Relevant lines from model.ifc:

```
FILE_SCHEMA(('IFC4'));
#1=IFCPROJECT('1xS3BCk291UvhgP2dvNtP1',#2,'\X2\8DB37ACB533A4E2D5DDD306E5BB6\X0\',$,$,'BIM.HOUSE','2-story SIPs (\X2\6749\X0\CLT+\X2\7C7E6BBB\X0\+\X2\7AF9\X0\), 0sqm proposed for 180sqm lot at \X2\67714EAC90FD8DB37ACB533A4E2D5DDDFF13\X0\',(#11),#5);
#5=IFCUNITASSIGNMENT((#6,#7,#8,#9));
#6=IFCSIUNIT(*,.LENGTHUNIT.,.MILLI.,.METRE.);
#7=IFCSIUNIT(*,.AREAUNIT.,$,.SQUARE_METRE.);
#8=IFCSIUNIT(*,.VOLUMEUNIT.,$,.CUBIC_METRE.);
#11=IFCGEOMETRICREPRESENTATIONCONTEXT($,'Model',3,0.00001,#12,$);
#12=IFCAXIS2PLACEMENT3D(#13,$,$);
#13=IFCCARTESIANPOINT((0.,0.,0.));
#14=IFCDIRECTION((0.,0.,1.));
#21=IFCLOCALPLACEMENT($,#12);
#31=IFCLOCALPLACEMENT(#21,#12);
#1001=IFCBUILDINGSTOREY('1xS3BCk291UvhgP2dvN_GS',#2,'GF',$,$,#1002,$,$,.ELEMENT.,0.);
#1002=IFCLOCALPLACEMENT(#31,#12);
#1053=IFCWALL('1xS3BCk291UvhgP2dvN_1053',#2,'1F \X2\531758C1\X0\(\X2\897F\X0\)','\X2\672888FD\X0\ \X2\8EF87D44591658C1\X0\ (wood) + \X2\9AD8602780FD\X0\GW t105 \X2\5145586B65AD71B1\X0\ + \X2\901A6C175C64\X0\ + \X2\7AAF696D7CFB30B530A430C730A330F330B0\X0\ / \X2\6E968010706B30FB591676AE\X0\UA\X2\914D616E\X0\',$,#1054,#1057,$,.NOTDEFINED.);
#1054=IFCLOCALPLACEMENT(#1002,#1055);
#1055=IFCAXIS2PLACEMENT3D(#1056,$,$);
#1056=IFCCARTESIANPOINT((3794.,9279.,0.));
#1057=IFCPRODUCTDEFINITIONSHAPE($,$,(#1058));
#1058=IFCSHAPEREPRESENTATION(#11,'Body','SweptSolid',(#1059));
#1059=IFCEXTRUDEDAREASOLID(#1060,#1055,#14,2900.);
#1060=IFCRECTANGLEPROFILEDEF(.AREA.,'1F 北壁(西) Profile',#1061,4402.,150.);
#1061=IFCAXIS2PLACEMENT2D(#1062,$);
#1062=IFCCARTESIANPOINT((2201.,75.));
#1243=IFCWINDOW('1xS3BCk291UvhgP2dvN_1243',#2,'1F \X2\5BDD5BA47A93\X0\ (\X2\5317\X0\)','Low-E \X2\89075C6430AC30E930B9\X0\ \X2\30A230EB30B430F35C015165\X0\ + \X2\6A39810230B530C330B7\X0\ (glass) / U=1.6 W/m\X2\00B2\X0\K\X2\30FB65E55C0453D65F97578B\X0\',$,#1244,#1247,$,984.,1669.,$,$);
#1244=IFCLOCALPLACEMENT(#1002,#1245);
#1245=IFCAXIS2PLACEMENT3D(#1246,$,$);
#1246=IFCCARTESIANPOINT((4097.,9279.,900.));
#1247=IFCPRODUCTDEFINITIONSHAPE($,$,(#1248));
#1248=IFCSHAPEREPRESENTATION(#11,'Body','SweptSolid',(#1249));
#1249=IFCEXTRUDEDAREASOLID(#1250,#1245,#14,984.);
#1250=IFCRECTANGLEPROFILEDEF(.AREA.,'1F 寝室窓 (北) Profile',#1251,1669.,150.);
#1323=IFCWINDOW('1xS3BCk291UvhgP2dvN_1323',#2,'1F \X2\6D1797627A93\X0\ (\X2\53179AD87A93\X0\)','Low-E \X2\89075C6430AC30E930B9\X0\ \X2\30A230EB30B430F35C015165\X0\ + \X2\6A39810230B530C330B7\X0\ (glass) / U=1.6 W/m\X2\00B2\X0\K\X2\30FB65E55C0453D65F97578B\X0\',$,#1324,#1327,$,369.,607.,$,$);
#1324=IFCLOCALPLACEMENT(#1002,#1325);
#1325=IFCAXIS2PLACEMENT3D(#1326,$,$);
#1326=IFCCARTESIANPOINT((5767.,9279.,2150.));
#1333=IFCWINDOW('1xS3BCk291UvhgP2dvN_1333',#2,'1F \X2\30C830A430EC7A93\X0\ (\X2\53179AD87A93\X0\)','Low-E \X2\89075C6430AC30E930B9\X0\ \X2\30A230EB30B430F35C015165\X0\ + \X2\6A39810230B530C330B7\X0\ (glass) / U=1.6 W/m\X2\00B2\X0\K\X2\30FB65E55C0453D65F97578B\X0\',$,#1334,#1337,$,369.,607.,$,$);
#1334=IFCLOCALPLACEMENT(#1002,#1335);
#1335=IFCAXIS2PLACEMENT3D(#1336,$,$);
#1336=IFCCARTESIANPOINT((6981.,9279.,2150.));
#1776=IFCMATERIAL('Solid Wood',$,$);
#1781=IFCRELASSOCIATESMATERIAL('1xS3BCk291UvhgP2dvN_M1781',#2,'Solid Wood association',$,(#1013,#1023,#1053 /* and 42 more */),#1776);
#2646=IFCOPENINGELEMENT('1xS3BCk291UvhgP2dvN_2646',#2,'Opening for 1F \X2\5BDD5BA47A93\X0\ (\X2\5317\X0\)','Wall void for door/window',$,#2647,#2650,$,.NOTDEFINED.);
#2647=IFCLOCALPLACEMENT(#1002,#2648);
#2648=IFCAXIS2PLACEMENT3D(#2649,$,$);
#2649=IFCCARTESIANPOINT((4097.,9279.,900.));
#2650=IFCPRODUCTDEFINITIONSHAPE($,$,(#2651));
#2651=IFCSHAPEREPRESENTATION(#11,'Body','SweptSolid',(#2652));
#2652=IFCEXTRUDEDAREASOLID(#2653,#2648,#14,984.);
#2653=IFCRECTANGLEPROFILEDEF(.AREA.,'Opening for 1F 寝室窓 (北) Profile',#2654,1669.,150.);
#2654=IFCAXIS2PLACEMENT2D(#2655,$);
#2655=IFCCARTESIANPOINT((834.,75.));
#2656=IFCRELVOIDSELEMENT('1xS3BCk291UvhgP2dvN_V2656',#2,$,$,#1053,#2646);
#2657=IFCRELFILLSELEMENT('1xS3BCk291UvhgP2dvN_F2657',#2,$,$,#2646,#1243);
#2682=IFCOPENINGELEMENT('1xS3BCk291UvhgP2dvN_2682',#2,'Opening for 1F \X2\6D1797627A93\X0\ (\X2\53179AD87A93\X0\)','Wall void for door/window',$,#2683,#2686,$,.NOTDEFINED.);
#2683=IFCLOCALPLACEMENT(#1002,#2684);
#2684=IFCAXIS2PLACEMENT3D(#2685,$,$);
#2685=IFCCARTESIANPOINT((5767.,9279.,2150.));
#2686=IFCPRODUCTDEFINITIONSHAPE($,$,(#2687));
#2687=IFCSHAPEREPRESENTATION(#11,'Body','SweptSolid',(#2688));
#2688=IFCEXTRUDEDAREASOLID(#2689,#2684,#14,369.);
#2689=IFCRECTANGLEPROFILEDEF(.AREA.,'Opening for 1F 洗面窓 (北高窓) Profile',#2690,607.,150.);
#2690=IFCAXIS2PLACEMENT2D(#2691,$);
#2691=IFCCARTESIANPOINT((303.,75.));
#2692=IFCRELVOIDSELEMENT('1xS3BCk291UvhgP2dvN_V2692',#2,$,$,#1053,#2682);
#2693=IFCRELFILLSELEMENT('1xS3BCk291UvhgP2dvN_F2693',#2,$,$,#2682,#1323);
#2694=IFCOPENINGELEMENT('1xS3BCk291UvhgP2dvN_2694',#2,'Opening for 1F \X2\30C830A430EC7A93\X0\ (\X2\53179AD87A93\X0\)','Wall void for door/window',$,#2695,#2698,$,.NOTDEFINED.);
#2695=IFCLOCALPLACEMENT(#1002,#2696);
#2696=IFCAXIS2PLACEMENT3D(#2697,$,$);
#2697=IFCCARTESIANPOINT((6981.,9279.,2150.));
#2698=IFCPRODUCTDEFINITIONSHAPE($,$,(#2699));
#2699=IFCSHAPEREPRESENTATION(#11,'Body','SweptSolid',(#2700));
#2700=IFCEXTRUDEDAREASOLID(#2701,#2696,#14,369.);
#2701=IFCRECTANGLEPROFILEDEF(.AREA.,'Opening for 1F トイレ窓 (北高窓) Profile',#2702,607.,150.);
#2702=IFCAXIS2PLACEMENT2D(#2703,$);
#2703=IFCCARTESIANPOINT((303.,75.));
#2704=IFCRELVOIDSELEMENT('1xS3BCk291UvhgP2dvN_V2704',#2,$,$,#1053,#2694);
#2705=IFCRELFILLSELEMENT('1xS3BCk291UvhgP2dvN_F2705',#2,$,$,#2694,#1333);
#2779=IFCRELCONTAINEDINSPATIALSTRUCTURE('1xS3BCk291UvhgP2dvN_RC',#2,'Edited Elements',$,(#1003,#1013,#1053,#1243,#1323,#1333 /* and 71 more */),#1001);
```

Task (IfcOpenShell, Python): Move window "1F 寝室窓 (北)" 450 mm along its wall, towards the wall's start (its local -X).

```python
import ifcopenshell
import ifcopenshell.api.geometry
import ifcopenshell.util.placement
import ifcopenshell.util.unit

model = ifcopenshell.open("model.ifc")
unit_scale = ifcopenshell.util.unit.calculate_unit_scale(model)

window = model.by_guid("1xS3BCk291UvhgP2dvN_1243")
opening = window.FillsVoids[0].RelatingOpeningElement
wall = opening.VoidsElements[0].RelatingBuildingElement

wall_matrix = ifcopenshell.util.placement.get_local_placement(wall.ObjectPlacement)
shift = wall_matrix[:3, 0] * -0.45 / unit_scale
before = ifcopenshell.util.placement.get_local_placement(window.ObjectPlacement)[:3, 3].copy()

# The window is not placed relative to its opening, so move both.
for product in (opening, window):
    matrix = ifcopenshell.util.placement.get_local_placement(product.ObjectPlacement)
    matrix[:3, 3] += shift
    ifcopenshell.api.geometry.edit_object_placement(model, product=product, matrix=matrix, is_si=False)

after = ifcopenshell.util.placement.get_local_placement(window.ObjectPlacement)[:3, 3]
print("window moved by", (after - before).round(3) + 0.0)

model.write("model_updated.ifc")
```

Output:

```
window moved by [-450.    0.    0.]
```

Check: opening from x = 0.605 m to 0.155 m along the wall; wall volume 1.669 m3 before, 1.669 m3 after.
